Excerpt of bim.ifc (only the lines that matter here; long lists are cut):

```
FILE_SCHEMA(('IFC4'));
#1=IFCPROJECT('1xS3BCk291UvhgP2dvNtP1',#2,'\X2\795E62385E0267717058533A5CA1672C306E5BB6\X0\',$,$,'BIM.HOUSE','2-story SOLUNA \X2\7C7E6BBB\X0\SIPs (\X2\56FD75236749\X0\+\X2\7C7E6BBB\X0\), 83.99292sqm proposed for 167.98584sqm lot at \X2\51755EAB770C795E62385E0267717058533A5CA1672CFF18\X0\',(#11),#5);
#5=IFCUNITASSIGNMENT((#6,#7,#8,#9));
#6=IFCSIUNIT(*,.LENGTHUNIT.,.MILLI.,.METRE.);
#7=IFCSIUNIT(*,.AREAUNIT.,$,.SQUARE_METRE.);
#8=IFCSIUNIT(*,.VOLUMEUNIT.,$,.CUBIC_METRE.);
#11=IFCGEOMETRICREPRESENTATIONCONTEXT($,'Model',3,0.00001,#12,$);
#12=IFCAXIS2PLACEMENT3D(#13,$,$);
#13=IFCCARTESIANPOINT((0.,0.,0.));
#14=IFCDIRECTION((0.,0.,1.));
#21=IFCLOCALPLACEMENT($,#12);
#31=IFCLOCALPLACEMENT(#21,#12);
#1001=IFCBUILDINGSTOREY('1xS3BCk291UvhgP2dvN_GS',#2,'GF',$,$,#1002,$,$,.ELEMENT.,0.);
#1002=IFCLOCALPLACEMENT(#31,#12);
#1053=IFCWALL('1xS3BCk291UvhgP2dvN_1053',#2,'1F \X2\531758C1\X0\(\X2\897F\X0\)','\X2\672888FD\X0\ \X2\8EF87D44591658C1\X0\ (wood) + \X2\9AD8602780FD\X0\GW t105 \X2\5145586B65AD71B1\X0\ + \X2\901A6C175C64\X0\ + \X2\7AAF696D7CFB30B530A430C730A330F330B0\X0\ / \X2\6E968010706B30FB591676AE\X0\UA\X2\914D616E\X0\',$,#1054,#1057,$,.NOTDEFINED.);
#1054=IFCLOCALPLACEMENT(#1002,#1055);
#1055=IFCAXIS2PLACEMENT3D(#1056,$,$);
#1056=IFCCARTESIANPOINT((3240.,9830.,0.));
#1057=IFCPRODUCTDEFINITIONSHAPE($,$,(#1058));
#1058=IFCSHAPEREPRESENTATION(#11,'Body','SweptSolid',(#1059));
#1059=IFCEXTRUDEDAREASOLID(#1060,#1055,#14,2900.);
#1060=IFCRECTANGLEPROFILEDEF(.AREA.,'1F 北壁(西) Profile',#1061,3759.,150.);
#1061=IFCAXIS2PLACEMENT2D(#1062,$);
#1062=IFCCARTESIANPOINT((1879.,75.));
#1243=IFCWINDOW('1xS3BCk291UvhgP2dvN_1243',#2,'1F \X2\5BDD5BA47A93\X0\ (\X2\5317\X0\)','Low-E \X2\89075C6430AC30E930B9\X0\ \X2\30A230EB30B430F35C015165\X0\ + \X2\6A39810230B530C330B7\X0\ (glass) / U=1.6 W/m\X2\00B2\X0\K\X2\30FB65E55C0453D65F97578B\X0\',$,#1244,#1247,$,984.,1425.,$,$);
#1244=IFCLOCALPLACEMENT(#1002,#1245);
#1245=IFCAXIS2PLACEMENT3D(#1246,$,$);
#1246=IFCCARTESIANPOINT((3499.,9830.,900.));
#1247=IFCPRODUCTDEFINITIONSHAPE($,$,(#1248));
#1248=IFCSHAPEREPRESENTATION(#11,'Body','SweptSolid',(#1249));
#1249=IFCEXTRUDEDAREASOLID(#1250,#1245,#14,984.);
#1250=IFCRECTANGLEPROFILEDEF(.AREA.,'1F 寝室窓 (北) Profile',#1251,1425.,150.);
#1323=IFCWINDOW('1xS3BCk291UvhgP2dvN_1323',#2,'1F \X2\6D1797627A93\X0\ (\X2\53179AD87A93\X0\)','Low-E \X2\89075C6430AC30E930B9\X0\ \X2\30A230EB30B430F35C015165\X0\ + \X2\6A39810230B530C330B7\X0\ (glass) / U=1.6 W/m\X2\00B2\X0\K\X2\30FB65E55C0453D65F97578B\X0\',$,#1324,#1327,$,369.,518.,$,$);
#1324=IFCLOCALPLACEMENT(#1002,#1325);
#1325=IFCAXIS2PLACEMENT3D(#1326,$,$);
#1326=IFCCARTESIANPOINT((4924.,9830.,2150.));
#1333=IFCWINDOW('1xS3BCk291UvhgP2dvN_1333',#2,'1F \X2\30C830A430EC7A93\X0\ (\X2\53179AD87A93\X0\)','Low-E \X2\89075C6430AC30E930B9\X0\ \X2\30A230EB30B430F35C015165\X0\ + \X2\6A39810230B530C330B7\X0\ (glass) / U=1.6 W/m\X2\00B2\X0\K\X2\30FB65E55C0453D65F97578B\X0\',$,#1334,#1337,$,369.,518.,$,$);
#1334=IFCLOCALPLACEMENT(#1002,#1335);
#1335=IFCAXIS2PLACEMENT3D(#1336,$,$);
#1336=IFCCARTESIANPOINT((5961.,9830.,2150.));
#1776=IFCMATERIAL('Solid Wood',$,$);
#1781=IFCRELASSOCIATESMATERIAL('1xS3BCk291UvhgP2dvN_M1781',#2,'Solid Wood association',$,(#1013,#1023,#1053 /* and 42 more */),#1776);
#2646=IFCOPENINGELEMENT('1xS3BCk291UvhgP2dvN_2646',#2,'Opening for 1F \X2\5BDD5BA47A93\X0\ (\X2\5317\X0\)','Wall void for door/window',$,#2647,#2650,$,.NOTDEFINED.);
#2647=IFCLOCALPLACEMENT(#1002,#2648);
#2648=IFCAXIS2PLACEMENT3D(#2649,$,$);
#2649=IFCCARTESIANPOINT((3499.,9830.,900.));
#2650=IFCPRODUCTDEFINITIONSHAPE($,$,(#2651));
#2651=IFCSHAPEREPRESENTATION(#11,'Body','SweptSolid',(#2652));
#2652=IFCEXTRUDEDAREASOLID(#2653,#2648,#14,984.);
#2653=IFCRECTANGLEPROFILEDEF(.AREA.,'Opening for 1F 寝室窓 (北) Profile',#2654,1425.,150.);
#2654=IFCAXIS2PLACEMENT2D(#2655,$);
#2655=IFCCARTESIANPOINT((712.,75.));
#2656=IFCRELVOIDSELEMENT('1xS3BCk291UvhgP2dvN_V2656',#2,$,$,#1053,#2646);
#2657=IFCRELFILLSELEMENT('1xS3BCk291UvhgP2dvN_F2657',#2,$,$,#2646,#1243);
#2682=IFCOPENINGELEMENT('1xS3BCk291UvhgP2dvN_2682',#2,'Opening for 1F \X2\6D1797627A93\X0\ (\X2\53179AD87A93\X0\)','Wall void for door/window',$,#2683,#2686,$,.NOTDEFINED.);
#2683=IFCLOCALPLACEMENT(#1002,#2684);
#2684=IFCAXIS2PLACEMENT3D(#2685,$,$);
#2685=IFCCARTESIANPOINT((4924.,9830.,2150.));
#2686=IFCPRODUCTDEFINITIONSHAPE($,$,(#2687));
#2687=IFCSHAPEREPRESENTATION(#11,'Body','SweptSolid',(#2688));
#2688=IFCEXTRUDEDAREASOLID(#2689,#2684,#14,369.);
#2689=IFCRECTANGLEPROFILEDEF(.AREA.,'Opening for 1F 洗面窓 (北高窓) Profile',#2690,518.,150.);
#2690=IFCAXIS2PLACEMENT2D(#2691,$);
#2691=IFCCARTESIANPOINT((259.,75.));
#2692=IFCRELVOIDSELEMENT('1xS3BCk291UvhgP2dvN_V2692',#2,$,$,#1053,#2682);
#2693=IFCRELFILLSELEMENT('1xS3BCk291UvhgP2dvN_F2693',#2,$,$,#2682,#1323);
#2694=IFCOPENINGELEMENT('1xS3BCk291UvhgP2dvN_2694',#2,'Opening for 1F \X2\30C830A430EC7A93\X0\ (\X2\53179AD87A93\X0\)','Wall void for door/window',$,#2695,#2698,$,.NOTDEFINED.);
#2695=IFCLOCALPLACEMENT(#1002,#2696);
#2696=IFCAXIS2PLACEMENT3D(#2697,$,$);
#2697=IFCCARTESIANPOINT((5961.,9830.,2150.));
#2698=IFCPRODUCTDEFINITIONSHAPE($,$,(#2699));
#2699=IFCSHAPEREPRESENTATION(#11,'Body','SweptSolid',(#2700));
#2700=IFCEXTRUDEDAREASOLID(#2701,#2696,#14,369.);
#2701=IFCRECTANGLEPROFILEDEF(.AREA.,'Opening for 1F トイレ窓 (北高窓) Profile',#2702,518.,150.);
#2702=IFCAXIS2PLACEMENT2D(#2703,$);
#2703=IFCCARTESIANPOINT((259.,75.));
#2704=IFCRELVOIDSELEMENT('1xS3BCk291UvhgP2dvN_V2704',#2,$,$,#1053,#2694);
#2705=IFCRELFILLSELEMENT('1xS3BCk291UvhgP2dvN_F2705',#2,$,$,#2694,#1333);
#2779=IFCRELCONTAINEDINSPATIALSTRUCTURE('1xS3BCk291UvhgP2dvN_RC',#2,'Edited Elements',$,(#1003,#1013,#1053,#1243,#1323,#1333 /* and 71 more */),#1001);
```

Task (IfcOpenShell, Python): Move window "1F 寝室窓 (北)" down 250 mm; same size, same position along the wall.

```python
import numpy as np
import ifcopenshell
import ifcopenshell.api.geometry
import ifcopenshell.util.placement
import ifcopenshell.util.unit

model = ifcopenshell.open("bim.ifc")
unit_scale = ifcopenshell.util.unit.calculate_unit_scale(model)

window = model.by_guid("1xS3BCk291UvhgP2dvN_1243")
opening = window.FillsVoids[0].RelatingOpeningElement
dz = -0.25 / unit_scale

shift = np.array([0.0, 0.0, dz])
# The window is not placed relative to its opening, so move both.
for product in (opening, window):
    matrix = ifcopenshell.util.placement.get_local_placement(product.ObjectPlacement)
    matrix[:3, 3] += shift
    ifcopenshell.api.geometry.edit_object_placement(model, product=product, matrix=matrix, is_si=False)

print(f"moved by {dz * unit_scale:+.3f} m")

model.write("bim_rev.ifc")
```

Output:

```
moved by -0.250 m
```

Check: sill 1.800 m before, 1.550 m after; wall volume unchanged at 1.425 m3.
